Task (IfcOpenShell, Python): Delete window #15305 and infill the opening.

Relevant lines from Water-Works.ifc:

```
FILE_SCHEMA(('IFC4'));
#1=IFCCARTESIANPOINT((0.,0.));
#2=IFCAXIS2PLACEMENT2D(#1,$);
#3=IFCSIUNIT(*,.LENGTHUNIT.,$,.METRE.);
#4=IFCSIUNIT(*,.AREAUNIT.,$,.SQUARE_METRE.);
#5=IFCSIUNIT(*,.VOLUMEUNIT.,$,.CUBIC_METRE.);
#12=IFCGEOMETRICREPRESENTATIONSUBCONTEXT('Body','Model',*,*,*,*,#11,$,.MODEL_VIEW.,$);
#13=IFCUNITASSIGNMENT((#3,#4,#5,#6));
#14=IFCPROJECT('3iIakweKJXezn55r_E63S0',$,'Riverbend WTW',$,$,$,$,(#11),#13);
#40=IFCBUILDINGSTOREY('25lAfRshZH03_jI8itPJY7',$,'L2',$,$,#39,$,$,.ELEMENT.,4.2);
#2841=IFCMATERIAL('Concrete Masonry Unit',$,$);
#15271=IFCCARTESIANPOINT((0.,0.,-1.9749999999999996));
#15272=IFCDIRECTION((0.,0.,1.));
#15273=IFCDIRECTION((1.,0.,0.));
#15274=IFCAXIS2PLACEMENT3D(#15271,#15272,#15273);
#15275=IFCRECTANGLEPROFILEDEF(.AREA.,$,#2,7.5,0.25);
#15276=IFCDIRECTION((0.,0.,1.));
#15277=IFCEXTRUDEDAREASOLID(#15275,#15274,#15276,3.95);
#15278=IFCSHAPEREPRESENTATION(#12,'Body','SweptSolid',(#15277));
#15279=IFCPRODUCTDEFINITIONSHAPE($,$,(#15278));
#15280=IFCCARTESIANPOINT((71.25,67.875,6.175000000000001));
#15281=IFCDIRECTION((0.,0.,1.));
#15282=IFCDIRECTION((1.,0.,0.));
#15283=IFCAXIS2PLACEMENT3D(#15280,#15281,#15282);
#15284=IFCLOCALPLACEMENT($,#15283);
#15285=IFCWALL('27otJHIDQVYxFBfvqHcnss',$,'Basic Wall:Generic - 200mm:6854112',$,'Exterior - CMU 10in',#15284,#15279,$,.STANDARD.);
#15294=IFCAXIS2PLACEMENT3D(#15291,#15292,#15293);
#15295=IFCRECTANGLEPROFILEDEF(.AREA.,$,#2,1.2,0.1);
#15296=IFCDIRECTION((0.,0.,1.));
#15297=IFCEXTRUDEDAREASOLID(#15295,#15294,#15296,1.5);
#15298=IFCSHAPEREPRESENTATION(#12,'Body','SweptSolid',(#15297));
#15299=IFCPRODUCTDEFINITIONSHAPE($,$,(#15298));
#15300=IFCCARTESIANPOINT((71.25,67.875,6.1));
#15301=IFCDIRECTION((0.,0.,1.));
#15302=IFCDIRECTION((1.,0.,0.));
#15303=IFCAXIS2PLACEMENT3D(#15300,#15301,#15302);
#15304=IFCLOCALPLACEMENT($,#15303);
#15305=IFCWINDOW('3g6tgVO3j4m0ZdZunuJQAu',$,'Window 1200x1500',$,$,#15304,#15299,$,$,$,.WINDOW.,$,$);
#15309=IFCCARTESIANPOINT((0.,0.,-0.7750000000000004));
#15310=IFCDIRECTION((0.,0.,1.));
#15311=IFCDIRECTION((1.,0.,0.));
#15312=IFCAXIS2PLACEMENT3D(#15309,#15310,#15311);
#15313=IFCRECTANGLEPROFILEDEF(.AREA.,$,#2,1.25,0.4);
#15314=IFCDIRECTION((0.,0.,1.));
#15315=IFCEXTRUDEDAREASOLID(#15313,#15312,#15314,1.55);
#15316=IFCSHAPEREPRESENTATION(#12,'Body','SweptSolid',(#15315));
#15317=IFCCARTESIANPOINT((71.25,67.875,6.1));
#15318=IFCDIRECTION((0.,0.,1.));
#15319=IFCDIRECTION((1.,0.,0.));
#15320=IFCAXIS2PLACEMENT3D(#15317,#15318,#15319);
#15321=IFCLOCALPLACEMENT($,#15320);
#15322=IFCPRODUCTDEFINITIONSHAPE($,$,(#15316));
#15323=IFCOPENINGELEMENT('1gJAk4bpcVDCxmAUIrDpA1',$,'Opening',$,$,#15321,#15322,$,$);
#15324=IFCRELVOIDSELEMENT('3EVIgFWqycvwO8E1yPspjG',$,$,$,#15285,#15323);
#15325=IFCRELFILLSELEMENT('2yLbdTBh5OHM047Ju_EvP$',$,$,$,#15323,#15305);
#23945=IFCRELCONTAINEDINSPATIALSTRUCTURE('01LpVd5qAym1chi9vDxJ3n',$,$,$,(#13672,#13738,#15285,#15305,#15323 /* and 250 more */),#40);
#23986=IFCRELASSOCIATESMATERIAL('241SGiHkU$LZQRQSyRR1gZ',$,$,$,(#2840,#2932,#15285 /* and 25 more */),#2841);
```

```python
import ifcopenshell
import ifcopenshell.api.feature
import ifcopenshell.api.root
import ifcopenshell.geom
import ifcopenshell.util.shape

model = ifcopenshell.open("Water-Works.ifc")
settings = ifcopenshell.geom.settings()


def volume(element):
    """Net volume in cubic metres, openings subtracted."""
    shape = ifcopenshell.geom.create_shape(settings, element)
    return ifcopenshell.util.shape.get_volume(shape.geometry)


window = model.by_guid("3g6tgVO3j4m0ZdZunuJQAu")
opening = window.FillsVoids[0].RelatingOpeningElement
wall = opening.VoidsElements[0].RelatingBuildingElement
before = volume(wall)

ifcopenshell.api.root.remove_product(model, product=window)
ifcopenshell.api.feature.remove_feature(model, feature=opening)

after = volume(wall)

print(f"wall volume {before:.3f} -> {after:.3f} m3")

model.write("Water-Works_edited.ifc")
```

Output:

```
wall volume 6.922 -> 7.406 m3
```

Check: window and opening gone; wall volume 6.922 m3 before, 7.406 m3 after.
